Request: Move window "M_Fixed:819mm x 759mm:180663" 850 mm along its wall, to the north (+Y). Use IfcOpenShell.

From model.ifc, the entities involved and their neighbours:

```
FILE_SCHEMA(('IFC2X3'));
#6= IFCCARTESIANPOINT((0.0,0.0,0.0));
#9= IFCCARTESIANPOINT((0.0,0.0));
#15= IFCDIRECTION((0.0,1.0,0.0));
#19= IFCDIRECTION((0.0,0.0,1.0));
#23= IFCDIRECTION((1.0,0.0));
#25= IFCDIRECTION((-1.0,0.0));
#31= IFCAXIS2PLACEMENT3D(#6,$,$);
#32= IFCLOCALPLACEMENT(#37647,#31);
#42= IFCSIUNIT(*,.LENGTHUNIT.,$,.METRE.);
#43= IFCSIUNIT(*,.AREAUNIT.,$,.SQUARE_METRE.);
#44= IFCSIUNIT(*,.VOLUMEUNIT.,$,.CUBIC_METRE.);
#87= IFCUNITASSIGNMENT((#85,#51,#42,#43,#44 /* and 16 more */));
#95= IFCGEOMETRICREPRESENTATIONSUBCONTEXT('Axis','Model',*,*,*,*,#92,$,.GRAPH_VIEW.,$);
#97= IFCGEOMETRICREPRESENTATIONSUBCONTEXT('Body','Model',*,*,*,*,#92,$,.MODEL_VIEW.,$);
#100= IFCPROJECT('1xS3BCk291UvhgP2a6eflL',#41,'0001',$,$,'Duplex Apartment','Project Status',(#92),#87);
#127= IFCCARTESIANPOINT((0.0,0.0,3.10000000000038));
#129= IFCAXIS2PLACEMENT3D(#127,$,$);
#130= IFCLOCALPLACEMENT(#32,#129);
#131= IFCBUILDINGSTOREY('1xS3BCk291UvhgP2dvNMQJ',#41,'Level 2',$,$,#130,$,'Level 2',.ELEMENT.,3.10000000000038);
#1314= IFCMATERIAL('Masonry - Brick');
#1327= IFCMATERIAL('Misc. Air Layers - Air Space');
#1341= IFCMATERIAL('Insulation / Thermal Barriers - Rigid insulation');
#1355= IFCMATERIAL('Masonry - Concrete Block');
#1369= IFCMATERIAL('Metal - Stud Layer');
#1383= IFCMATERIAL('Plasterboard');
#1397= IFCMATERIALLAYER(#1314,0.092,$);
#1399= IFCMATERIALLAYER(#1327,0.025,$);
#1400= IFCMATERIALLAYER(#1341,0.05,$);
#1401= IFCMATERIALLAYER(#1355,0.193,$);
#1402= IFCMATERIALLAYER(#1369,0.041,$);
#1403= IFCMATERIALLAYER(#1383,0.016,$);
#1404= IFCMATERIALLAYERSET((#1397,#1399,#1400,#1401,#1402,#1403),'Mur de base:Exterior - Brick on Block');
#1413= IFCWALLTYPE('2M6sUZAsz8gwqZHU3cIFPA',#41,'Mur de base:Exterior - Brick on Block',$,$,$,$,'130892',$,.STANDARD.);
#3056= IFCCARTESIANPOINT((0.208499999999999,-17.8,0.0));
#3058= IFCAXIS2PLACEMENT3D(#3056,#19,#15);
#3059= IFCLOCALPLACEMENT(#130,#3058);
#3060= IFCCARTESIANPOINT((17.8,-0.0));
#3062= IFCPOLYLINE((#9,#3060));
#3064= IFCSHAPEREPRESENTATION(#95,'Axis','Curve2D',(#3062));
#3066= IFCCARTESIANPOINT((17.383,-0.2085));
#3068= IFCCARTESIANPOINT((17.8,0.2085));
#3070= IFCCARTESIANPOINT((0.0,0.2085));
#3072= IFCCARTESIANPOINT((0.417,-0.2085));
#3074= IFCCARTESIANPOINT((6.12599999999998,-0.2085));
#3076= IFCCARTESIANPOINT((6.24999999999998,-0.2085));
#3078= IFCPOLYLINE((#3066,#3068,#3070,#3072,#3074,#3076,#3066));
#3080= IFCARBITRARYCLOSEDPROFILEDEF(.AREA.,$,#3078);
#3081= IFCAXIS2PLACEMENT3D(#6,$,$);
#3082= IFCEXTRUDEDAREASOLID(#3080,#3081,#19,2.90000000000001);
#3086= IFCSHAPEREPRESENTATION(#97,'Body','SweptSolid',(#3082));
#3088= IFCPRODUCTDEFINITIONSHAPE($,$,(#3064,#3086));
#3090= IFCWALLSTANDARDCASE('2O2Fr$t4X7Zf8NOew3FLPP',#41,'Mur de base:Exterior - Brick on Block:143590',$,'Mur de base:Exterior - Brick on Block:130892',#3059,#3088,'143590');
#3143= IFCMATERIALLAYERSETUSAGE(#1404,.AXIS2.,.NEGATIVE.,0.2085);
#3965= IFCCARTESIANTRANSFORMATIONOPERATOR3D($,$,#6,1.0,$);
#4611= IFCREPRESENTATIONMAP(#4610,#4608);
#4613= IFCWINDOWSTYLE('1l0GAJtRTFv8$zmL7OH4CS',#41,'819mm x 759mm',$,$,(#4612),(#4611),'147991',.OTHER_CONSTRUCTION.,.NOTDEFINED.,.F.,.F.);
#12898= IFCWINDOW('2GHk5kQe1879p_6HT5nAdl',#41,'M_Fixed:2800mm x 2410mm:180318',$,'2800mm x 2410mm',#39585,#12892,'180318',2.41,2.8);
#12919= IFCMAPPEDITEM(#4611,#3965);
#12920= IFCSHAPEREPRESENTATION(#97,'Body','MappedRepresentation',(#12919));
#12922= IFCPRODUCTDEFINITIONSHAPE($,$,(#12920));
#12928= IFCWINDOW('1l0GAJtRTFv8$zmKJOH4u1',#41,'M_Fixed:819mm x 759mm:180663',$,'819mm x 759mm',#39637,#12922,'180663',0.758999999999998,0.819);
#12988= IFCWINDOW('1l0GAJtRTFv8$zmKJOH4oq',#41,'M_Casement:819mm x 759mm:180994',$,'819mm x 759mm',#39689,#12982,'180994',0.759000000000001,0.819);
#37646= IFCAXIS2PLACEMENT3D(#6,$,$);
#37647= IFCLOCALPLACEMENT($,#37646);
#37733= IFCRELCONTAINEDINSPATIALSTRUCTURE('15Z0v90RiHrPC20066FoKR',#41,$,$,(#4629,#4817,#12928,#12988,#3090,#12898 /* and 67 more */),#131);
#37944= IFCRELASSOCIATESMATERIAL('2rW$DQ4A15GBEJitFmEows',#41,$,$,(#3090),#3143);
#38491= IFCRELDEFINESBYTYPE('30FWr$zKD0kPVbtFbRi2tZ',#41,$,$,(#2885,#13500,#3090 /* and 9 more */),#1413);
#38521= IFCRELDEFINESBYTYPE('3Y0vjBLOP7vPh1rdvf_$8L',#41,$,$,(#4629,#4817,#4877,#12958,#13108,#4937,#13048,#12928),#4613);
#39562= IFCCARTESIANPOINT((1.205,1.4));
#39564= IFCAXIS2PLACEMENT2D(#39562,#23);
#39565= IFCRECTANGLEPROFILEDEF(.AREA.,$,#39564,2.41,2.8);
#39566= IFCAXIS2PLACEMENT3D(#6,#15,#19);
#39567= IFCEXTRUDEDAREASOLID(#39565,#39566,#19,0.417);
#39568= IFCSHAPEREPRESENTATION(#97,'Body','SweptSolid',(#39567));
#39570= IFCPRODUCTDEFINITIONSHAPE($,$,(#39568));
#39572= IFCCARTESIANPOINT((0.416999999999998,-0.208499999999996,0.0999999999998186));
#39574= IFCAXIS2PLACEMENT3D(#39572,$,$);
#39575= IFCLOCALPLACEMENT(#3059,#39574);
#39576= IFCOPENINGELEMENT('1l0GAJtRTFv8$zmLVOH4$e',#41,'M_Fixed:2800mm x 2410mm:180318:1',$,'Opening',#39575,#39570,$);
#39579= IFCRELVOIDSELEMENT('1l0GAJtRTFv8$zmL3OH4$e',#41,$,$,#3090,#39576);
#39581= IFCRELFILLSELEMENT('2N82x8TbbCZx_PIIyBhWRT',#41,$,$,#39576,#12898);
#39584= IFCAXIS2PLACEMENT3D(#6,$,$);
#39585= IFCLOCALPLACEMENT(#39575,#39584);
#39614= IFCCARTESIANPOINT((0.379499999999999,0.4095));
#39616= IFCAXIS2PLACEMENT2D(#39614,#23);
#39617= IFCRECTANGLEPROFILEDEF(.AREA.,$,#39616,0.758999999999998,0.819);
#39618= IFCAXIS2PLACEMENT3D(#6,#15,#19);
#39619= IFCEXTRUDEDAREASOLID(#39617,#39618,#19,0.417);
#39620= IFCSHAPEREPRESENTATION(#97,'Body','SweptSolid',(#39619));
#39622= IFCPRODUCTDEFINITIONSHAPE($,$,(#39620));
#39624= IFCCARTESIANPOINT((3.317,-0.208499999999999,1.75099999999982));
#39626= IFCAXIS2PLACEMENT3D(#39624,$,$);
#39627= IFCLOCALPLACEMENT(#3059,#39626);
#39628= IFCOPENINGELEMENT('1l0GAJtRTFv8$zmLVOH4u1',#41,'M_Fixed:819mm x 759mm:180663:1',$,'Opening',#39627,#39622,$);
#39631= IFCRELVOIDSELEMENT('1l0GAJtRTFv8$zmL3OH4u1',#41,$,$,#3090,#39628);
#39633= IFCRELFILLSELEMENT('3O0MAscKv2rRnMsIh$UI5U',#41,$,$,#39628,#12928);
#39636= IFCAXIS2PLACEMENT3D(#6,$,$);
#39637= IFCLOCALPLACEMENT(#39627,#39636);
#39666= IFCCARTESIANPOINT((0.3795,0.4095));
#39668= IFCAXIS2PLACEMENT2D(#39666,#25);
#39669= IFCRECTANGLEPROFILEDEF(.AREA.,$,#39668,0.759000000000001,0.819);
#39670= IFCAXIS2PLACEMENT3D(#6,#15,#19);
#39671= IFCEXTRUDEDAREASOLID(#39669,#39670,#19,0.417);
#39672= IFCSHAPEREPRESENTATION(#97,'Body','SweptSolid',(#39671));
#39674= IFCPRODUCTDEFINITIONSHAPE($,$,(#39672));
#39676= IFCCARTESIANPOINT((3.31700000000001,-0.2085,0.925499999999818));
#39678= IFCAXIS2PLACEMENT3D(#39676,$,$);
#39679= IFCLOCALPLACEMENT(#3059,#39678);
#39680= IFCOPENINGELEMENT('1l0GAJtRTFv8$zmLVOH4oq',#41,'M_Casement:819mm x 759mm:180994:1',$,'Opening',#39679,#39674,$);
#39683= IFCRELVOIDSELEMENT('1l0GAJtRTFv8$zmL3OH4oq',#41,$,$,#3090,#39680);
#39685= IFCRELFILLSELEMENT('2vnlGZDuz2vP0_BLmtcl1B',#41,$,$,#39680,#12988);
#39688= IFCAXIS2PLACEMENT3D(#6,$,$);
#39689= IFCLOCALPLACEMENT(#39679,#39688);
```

```python
import ifcopenshell
import ifcopenshell.api.geometry
import ifcopenshell.util.placement

model = ifcopenshell.open("model.ifc")

window = model.by_id(12928)
opening = window.FillsVoids[0].RelatingOpeningElement
wall = opening.VoidsElements[0].RelatingBuildingElement

wall_matrix = ifcopenshell.util.placement.get_local_placement(wall.ObjectPlacement)
shift = wall_matrix[:3, 0] * 0.85
before = ifcopenshell.util.placement.get_local_placement(window.ObjectPlacement)[:3, 3].copy()

# The window is placed relative to its opening, so it follows when the opening moves.
matrix = ifcopenshell.util.placement.get_local_placement(opening.ObjectPlacement)
matrix[:3, 3] += shift
ifcopenshell.api.geometry.edit_object_placement(
    model, product=opening, matrix=matrix, is_si=False, should_transform_children=True
)

after = ifcopenshell.util.placement.get_local_placement(window.ObjectPlacement)[:3, 3]
print("window moved by", (after - before).round(3) + 0.0)

model.write("model_rev.ifc")
```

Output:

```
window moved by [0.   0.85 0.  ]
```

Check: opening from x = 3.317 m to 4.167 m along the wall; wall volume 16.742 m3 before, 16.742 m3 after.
